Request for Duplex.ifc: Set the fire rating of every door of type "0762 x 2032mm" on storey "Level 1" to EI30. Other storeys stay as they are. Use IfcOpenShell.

First a look at what the model holds.

```python
import ifcopenshell
import ifcopenshell.util.element

model = ifcopenshell.open("Duplex.ifc")
print(model.schema)
storey = next(s for s in model.by_type("IfcBuildingStorey") if s.Name == "Level 1")
doors = [e for e in ifcopenshell.util.element.get_decomposition(storey) if e.is_a("IfcDoor")]
seen = {}
for e in doors:
    element_type = ifcopenshell.util.element.get_type(e)
    key = (element_type.Name if element_type != e and element_type else None, ifcopenshell.util.element.get_pset(e, "Pset_DoorCommon", "FireRating"))
    seen[key] = seen.get(key, 0) + 1
for (name, value), count in sorted(seen.items(), key=str):
    print(count, "x", name, "|", value)
```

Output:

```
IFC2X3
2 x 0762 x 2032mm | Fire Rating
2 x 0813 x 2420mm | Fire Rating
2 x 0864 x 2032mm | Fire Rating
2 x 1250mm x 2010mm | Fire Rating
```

```python
import ifcopenshell
import ifcopenshell.api.pset
import ifcopenshell.util.element

model = ifcopenshell.open("Duplex.ifc")

storey = next(s for s in model.by_type("IfcBuildingStorey") if s.Name == "Level 1")
doors = [e for e in ifcopenshell.util.element.get_decomposition(storey) if e.is_a("IfcDoor")]

count = 0
for e in doors:
    element_type = ifcopenshell.util.element.get_type(e)
    if element_type in (None, e) or element_type.Name != "0762 x 2032mm":
        continue
    # add_pset returns the element's existing set when there is one.
    pset = ifcopenshell.api.pset.add_pset(model, product=e, name="Pset_DoorCommon")
    ifcopenshell.api.pset.edit_pset(model, pset=pset, properties={"FireRating": "EI30"})
    count += 1

print(count, "doors updated")

model.write("Duplex_updated.ifc")
```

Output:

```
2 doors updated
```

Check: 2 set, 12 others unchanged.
